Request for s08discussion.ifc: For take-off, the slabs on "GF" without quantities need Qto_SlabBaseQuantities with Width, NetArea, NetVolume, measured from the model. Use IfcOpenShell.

First a look at what the model holds.

```python
import ifcopenshell
import ifcopenshell.util.element
import ifcopenshell.util.unit

model = ifcopenshell.open("s08discussion.ifc")
print(model.schema)
for unit_type in ("LENGTHUNIT", "AREAUNIT", "VOLUMEUNIT"):
    print(unit_type, ifcopenshell.util.unit.calculate_unit_scale(model, unit_type))
storey = next(s for s in model.by_type("IfcBuildingStorey") if s.Name == "GF")
slabs = [e for e in ifcopenshell.util.element.get_decomposition(storey) if e.is_a("IfcSlab")]
for e in sorted(slabs, key=lambda e: e.id()):
    print(e.id(), e.is_a(), e.Name, list(ifcopenshell.util.element.get_psets(e, qtos_only=True)), sep=" | ")
```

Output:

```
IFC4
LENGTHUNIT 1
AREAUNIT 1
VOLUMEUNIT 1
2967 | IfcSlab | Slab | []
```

```python
import ifcopenshell
import ifcopenshell.api.pset
import ifcopenshell.geom
import ifcopenshell.util.element
import ifcopenshell.util.shape
import ifcopenshell.util.unit

model = ifcopenshell.open("s08discussion.ifc")
unit_scale = ifcopenshell.util.unit.calculate_unit_scale(model)
area_scale = ifcopenshell.util.unit.calculate_unit_scale(model, "AREAUNIT")
volume_scale = ifcopenshell.util.unit.calculate_unit_scale(model, "VOLUMEUNIT")
settings = ifcopenshell.geom.settings()

storey = next(s for s in model.by_type("IfcBuildingStorey") if s.Name == "GF")
slabs = [e for e in ifcopenshell.util.element.get_decomposition(storey) if e.is_a("IfcSlab")]

for e in sorted(slabs, key=lambda e: e.id()):
    if ifcopenshell.util.element.get_psets(e, qtos_only=True, should_inherit=False):
        continue
    # Geometry comes back in metres, in the element's own axes.
    shape = ifcopenshell.geom.create_shape(settings, e)
    values = {
        "Width": ifcopenshell.util.shape.get_z(shape.geometry) / unit_scale,
        "NetArea": ifcopenshell.util.shape.get_footprint_area(shape.geometry) / area_scale,
        "NetVolume": ifcopenshell.util.shape.get_volume(shape.geometry) / volume_scale,
    }
    qto = ifcopenshell.api.pset.add_qto(model, product=e, name="Qto_SlabBaseQuantities")
    ifcopenshell.api.pset.edit_qto(model, qto=qto, properties=values)
    print(e.id(), {k: round(v, 3) for k, v in values.items()})

model.write("s08discussion_edited.ifc")
```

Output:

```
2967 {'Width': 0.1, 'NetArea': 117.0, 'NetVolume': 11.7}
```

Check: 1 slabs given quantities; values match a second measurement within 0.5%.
